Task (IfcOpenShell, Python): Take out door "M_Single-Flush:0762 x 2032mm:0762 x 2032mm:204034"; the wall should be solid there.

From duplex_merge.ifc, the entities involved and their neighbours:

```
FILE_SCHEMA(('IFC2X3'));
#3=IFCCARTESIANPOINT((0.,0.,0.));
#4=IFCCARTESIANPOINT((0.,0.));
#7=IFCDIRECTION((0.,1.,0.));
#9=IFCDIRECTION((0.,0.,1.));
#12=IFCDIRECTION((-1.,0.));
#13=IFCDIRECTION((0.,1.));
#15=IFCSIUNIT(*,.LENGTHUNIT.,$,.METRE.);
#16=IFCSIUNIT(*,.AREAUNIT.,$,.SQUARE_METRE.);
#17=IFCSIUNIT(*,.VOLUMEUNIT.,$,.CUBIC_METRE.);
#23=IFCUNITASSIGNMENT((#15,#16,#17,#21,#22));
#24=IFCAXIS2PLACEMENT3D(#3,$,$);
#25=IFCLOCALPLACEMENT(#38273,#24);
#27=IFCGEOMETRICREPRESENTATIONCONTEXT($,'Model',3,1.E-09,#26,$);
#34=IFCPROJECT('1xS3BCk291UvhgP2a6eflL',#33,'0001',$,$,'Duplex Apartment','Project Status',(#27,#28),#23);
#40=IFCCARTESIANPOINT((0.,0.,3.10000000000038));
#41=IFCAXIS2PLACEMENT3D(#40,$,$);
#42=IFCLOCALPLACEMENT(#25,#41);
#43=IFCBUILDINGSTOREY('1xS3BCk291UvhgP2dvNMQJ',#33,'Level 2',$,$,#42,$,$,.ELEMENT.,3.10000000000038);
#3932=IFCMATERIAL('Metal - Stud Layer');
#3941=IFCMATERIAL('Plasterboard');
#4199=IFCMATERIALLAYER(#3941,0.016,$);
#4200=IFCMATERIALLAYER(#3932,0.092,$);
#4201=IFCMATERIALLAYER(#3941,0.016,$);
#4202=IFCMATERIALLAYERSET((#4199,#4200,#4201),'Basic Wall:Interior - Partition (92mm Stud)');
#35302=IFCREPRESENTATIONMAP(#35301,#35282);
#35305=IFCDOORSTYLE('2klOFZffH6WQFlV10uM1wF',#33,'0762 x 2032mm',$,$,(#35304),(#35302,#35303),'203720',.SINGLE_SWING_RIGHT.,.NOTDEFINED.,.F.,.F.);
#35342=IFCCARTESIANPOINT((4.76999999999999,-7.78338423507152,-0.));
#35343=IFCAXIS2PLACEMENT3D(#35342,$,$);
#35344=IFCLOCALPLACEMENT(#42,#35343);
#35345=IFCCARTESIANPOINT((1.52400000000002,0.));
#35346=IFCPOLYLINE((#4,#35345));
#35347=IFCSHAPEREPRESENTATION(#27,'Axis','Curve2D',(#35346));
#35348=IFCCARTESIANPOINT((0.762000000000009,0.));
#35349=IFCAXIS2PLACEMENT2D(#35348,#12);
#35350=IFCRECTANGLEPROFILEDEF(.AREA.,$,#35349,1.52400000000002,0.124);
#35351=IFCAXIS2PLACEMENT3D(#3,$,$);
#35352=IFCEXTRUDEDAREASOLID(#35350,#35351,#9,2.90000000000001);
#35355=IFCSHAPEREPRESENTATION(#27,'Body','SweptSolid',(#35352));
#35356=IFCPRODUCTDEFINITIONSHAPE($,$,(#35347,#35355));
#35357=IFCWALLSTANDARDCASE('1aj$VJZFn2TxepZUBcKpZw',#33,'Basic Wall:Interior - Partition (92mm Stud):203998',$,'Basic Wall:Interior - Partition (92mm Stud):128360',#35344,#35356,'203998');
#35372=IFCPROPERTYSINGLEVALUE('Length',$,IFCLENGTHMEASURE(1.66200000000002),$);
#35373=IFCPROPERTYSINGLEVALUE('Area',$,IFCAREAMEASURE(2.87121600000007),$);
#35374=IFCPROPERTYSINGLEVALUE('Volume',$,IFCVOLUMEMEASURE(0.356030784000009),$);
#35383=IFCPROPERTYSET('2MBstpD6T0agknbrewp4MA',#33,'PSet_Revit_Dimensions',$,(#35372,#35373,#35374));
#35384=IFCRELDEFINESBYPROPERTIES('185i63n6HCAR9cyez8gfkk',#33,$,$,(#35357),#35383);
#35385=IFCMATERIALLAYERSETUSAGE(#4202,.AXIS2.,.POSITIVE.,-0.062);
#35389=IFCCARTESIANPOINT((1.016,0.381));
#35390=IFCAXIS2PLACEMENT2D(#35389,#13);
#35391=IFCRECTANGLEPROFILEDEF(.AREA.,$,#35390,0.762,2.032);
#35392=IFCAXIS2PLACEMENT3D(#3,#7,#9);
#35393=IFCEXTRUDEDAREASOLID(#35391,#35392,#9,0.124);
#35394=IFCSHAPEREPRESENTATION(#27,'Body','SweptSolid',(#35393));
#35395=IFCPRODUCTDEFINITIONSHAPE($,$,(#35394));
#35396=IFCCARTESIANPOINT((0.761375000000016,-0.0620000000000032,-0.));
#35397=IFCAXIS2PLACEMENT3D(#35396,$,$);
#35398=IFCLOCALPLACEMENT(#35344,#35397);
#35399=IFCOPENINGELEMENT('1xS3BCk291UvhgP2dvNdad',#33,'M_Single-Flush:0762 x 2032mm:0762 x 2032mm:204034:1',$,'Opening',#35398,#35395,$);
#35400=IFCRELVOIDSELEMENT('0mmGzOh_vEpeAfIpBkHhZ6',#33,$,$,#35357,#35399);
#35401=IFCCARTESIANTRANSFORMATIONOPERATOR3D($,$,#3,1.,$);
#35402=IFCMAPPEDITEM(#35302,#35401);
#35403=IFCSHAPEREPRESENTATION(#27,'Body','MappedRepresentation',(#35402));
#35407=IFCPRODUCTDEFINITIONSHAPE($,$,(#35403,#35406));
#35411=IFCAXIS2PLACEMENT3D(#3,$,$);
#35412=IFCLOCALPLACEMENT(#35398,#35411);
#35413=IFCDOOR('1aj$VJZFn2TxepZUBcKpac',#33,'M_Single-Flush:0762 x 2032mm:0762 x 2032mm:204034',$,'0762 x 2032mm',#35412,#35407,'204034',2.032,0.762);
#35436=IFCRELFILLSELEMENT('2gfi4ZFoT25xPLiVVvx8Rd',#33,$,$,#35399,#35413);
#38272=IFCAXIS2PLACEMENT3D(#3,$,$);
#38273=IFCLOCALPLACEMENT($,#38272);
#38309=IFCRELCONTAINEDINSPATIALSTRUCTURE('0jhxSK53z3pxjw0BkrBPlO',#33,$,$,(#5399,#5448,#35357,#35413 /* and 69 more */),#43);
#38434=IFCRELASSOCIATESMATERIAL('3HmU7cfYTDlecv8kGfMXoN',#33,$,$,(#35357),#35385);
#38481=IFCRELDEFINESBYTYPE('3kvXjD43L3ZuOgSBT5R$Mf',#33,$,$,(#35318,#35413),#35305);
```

```python
import ifcopenshell
import ifcopenshell.api.feature
import ifcopenshell.api.pset
import ifcopenshell.api.root
import ifcopenshell.geom
import ifcopenshell.util.element
import ifcopenshell.util.shape
import ifcopenshell.util.unit

model = ifcopenshell.open("duplex_merge.ifc")
area_scale = ifcopenshell.util.unit.calculate_unit_scale(model, "AREAUNIT")
volume_scale = ifcopenshell.util.unit.calculate_unit_scale(model, "VOLUMEUNIT")
settings = ifcopenshell.geom.settings()


def volume(element):
    """Net volume in cubic metres, openings subtracted."""
    shape = ifcopenshell.geom.create_shape(settings, element)
    return ifcopenshell.util.shape.get_volume(shape.geometry)


door = model.by_guid("1aj$VJZFn2TxepZUBcKpac")
opening = door.FillsVoids[0].RelatingOpeningElement
wall = opening.VoidsElements[0].RelatingBuildingElement
before = volume(wall)

ifcopenshell.api.root.remove_product(model, product=door)
ifcopenshell.api.feature.remove_feature(model, feature=opening)

after = volume(wall)
thickness = 0.124  # wall thickness in metres

# Update the wall's stored quantities.
pset = model.by_id(ifcopenshell.util.element.get_pset(wall, "PSet_Revit_Dimensions", should_inherit=False)["id"])
ifcopenshell.api.pset.edit_pset(model, pset=pset, properties={
    "Area": model.create_entity("IfcAreaMeasure", after / thickness / area_scale),
    "Volume": model.create_entity("IfcVolumeMeasure", after / volume_scale),
})

print(f"wall volume {before:.3f} -> {after:.3f} m3")

model.write("duplex_merge-out.ifc")
```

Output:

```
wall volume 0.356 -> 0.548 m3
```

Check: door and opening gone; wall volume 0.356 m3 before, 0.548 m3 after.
